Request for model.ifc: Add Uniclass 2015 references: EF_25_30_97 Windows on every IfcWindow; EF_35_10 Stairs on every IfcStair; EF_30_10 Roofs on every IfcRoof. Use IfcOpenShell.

First a look at what the model holds.

```python
import ifcopenshell

model = ifcopenshell.open("model.ifc")
print(model.schema)
print("classifications:", [c.Name for c in model.by_type("IfcClassification")])
for ifc_class in ("IfcDoor", "IfcRoof", "IfcStair", "IfcWall", "IfcWindow"):
    print(ifc_class, len(model.by_type(ifc_class)))
```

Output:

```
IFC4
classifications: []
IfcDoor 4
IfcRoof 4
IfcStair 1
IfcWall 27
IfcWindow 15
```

```python
import ifcopenshell
import ifcopenshell.api.classification

model = ifcopenshell.open("model.ifc")

system = ifcopenshell.api.classification.add_classification(model, classification="Uniclass 2015")

codes = {
    "IfcWindow": ("EF_25_30_97", "Windows"),
    "IfcStair": ("EF_35_10", "Stairs"),
    "IfcRoof": ("EF_30_10", "Roofs"),
}
for ifc_class, (code, name) in codes.items():
    products = model.by_type(ifc_class)
    ifcopenshell.api.classification.add_reference(
        model, products=products, classification=system, identification=code, name=name
    )
    print(code, len(products))

model.write("model_edited.ifc")
```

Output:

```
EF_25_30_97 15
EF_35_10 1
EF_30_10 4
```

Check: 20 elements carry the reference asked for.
